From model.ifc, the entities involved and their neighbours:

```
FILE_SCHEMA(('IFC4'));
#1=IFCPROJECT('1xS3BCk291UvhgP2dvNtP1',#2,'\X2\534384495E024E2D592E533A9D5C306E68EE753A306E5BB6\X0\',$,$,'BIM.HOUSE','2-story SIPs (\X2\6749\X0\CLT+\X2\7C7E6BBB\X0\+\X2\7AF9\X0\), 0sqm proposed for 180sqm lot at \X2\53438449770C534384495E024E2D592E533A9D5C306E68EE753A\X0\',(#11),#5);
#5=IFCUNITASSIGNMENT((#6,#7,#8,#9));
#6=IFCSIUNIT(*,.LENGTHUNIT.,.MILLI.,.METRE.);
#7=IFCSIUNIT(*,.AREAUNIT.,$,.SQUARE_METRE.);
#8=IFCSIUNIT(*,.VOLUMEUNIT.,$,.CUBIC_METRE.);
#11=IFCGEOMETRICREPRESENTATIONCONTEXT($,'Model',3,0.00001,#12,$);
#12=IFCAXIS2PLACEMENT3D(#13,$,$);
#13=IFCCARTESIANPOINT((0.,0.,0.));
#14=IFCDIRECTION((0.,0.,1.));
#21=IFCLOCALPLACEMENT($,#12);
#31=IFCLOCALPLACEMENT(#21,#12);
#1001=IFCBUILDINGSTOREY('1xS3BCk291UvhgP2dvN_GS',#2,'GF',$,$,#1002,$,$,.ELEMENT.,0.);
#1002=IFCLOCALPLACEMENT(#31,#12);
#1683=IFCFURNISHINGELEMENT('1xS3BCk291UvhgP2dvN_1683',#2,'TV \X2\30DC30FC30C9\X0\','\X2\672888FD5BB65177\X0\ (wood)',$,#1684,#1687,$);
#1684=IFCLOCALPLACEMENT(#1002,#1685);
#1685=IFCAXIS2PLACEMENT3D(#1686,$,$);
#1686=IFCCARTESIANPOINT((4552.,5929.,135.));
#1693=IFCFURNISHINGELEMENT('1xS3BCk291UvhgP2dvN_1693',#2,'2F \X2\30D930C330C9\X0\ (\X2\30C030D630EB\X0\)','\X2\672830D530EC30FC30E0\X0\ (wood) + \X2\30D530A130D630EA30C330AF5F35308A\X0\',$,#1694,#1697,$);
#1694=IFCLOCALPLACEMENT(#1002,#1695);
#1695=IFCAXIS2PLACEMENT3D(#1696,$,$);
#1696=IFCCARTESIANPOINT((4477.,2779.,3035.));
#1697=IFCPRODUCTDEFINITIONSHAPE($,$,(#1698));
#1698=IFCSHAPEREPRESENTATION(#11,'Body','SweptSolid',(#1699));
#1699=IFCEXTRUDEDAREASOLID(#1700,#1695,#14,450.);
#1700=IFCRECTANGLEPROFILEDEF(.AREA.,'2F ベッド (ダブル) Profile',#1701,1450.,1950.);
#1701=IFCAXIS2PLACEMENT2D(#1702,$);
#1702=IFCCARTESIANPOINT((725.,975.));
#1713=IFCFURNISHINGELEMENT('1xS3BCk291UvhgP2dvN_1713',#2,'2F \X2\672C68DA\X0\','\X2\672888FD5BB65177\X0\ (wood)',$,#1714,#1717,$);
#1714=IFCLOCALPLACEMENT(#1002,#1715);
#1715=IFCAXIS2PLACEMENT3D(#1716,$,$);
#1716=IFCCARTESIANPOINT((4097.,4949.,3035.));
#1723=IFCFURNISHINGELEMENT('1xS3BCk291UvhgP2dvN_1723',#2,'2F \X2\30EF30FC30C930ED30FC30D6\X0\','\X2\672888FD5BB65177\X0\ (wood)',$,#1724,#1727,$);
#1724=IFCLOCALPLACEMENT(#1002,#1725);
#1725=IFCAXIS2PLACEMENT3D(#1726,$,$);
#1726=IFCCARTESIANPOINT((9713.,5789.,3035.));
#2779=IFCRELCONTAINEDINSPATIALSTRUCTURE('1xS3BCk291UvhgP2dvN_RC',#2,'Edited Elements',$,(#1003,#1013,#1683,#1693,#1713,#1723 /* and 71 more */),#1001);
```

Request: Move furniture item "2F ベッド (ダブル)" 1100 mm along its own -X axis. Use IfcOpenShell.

```python
import ifcopenshell
import ifcopenshell.api.geometry
import ifcopenshell.util.placement

model = ifcopenshell.open("model.ifc")

item = model.by_guid("1xS3BCk291UvhgP2dvN_1693")
matrix = ifcopenshell.util.placement.get_local_placement(item.ObjectPlacement)
matrix[:3, 3] -= matrix[:3, 0] * 1100.0
ifcopenshell.api.geometry.edit_object_placement(model, product=item, matrix=matrix, is_si=False)

print(ifcopenshell.util.placement.get_local_placement(item.ObjectPlacement).round(3) + 0.0)

model.write("model-out.ifc")
```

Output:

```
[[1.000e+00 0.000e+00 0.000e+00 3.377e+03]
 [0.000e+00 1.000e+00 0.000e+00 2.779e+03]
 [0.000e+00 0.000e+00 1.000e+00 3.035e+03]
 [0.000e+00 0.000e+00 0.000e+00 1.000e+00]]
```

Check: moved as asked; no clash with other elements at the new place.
